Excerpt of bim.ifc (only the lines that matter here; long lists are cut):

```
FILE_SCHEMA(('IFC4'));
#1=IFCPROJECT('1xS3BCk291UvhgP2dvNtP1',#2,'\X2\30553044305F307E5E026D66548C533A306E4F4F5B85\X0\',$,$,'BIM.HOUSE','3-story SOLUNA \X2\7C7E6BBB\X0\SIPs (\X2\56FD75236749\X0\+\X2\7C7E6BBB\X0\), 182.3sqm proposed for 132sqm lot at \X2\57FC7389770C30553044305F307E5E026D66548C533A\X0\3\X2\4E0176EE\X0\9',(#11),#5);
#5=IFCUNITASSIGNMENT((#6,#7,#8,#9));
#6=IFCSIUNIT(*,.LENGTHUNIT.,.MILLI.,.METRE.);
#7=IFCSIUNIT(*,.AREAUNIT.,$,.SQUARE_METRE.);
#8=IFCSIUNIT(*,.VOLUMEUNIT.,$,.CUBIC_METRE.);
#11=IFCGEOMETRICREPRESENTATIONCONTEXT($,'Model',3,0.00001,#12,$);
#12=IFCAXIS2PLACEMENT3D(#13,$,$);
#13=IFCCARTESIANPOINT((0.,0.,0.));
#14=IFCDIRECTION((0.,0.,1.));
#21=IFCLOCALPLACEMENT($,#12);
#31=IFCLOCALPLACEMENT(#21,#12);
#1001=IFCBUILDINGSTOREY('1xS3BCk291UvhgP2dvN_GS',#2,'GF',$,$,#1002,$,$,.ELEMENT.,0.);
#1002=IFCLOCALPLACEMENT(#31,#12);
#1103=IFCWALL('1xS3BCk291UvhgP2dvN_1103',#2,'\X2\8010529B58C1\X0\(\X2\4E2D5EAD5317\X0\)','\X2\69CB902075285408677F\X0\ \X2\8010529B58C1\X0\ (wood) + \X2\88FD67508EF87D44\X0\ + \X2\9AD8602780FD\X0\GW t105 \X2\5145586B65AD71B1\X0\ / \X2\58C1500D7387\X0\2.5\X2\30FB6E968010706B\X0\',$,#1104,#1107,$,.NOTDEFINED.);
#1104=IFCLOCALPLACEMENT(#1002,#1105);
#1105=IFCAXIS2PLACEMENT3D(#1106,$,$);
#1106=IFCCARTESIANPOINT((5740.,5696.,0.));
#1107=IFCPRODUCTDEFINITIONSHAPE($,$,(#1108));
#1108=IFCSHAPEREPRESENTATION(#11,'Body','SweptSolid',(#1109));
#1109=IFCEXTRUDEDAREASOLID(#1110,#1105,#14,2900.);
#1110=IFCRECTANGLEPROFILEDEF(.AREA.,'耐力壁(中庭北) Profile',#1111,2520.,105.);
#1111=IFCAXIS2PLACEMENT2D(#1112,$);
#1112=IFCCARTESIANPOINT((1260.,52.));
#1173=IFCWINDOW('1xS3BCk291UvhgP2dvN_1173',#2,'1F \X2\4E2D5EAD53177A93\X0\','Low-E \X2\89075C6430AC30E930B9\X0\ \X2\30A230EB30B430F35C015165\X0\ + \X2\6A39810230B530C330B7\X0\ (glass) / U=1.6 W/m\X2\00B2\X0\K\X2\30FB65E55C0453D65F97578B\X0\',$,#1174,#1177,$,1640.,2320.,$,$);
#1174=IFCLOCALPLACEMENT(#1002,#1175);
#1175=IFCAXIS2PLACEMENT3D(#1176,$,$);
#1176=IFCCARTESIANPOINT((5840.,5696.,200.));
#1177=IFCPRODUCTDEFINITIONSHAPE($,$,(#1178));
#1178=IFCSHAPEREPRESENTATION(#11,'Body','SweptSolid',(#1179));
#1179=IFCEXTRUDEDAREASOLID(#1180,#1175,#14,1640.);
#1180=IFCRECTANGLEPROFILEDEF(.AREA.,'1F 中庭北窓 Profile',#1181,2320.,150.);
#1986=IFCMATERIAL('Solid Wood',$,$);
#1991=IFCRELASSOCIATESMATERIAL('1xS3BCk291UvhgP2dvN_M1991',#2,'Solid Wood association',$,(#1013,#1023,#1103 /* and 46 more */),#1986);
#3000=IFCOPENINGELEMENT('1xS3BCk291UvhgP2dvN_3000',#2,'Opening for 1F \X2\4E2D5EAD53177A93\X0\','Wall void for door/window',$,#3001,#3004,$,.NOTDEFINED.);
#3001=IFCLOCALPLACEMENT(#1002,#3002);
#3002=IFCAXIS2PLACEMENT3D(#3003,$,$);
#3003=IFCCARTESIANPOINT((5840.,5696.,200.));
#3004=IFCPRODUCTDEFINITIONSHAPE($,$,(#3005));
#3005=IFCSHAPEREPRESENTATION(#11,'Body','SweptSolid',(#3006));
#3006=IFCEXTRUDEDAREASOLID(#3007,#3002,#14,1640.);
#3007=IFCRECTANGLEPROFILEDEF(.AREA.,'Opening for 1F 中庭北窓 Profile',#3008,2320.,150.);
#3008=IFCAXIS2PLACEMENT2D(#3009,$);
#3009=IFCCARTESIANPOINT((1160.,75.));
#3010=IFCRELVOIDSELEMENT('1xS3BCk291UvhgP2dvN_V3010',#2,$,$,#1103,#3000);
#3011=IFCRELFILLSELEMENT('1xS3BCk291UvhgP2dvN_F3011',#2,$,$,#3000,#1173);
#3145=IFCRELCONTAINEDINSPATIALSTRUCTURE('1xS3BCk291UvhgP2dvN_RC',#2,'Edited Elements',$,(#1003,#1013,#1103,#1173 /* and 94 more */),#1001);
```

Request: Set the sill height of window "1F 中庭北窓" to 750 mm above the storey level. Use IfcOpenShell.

```python
import numpy as np
import ifcopenshell
import ifcopenshell.api.geometry
import ifcopenshell.geom
import ifcopenshell.util.element
import ifcopenshell.util.placement
import ifcopenshell.util.shape
import ifcopenshell.util.unit

model = ifcopenshell.open("bim.ifc")
unit_scale = ifcopenshell.util.unit.calculate_unit_scale(model)

window = model.by_id(1173)
opening = window.FillsVoids[0].RelatingOpeningElement
storey = ifcopenshell.util.element.get_container(window, ifc_class="IfcBuildingStorey")
level = ifcopenshell.util.placement.get_local_placement(storey.ObjectPlacement)[2, 3]

# The opening's origin need not be at the sill, so measure its lowest point.
shape = ifcopenshell.geom.create_shape(ifcopenshell.geom.settings(), opening)
bottom = ifcopenshell.util.shape.get_shape_bottom_elevation(shape, shape.geometry) / unit_scale
dz = level + 0.75 / unit_scale - bottom

shift = np.array([0.0, 0.0, dz])
# The window is not placed relative to its opening, so move both.
for product in (opening, window):
    matrix = ifcopenshell.util.placement.get_local_placement(product.ObjectPlacement)
    matrix[:3, 3] += shift
    ifcopenshell.api.geometry.edit_object_placement(model, product=product, matrix=matrix, is_si=False)

print(f"moved by {dz * unit_scale:+.3f} m")

model.write("bim-out.ifc")
```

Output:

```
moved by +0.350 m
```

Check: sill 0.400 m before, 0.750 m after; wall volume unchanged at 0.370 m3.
